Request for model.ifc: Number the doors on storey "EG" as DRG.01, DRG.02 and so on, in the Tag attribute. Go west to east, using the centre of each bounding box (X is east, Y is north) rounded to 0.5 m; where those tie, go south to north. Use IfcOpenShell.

First a look at what the model holds.

```python
import ifcopenshell
import ifcopenshell.util.element
import ifcopenshell.util.placement

model = ifcopenshell.open("model.ifc")
print(model.schema)
storey = next(s for s in model.by_type("IfcBuildingStorey") if s.Name == "EG")
doors = [e for e in ifcopenshell.util.element.get_decomposition(storey) if e.is_a("IfcDoor")]
for e in sorted(doors, key=lambda e: e.id()):
    origin = ifcopenshell.util.placement.get_local_placement(e.ObjectPlacement)[:3, 3]
    print(e.id(), e.Tag, e.Name, origin.round(2) + 0.0, sep=" | ")
```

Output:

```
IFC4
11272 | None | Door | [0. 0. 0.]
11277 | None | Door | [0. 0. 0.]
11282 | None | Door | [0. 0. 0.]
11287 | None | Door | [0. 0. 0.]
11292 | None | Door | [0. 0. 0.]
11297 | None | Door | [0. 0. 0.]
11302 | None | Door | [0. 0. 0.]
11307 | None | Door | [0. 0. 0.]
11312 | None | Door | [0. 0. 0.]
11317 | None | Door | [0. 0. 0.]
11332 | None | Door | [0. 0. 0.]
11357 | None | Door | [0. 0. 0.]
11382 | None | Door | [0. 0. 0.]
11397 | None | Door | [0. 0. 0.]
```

```python
import ifcopenshell
import ifcopenshell.geom
import ifcopenshell.util.element
import ifcopenshell.util.shape

model = ifcopenshell.open("model.ifc")
settings = ifcopenshell.geom.settings()
settings.set("use-world-coords", True)


def centre(element):
    shape = ifcopenshell.geom.create_shape(settings, element)
    return ifcopenshell.util.shape.get_bbox_centroid(shape.geometry)


storey = next(s for s in model.by_type("IfcBuildingStorey") if s.Name == "EG")
doors = [e for e in ifcopenshell.util.element.get_decomposition(storey) if e.is_a("IfcDoor")]

# Insertion points can sit at a corner or the storey origin, so sort by the geometry (in metres).
centres = {e: centre(e) for e in doors}
doors.sort(key=lambda e: (round(centres[e][0] / 0.5), centres[e][1]))

for i, e in enumerate(doors, start=1):
    number = f"DRG.{i:02d}"
    e.Tag = number
    print(e.id(), number)

model.write("model_v2.ifc")
```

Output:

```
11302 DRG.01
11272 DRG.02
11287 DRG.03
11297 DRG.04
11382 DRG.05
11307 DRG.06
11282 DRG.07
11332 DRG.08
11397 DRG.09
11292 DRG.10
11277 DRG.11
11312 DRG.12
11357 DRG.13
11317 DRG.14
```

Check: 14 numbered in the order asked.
